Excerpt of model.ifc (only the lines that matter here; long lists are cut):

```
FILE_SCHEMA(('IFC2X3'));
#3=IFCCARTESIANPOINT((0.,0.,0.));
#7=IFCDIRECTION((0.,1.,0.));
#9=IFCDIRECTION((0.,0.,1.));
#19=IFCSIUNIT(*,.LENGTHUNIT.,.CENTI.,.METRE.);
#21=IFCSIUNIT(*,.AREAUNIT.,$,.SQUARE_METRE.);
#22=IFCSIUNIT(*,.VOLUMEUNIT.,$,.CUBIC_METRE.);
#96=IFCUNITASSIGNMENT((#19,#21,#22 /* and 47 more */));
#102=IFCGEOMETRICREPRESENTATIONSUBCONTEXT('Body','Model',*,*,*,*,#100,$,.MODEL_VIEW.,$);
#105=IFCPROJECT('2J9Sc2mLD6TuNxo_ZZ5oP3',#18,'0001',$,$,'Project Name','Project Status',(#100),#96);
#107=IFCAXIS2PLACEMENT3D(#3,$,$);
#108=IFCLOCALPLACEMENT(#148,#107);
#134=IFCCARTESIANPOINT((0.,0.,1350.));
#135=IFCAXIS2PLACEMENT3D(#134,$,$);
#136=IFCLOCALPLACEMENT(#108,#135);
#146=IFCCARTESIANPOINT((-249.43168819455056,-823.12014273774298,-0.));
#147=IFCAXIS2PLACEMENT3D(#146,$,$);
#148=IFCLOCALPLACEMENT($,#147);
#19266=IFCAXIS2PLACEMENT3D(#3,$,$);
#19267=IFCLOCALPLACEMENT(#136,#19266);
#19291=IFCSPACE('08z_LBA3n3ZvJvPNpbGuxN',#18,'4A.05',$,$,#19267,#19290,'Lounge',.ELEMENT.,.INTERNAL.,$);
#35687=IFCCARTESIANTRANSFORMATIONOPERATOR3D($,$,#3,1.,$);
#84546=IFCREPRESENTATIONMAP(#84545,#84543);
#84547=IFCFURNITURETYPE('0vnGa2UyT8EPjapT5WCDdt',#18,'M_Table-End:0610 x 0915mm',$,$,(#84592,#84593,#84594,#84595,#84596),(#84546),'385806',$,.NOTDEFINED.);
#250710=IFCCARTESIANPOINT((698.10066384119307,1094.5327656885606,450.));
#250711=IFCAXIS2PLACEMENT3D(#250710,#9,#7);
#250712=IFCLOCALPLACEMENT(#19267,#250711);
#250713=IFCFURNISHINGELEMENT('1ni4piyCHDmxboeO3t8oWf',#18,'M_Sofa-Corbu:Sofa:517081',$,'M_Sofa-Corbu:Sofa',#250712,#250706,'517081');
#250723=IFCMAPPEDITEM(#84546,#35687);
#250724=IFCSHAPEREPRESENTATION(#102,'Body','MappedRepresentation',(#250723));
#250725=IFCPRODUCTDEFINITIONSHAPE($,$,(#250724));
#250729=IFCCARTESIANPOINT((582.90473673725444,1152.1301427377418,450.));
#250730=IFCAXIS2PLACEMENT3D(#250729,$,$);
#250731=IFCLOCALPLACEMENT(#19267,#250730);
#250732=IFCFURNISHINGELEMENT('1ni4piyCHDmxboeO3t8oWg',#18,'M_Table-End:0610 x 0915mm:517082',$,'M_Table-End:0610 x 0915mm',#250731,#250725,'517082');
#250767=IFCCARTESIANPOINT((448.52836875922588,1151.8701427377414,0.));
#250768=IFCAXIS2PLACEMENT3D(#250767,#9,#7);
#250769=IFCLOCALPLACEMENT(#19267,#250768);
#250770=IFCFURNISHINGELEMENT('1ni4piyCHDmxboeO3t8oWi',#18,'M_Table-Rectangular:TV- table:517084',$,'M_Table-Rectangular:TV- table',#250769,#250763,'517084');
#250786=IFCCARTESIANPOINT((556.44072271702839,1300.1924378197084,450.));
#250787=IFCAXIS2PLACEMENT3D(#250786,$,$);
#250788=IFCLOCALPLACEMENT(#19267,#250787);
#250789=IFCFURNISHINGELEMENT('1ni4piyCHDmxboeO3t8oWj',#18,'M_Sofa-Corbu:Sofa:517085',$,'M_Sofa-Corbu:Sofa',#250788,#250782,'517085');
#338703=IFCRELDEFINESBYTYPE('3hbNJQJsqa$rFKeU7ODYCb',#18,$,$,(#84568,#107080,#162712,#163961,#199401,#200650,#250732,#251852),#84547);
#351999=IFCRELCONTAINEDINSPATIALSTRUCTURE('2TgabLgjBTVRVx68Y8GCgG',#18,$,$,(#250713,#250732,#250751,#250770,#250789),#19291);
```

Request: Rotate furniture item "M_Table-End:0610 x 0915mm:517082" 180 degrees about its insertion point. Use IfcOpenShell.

```python
import ifcopenshell
import ifcopenshell.api.geometry
import ifcopenshell.util.placement

model = ifcopenshell.open("model.ifc")

item = model.by_guid("1ni4piyCHDmxboeO3t8oWg")
matrix = ifcopenshell.util.placement.get_local_placement(item.ObjectPlacement)
matrix = matrix @ ifcopenshell.util.placement.rotation(180, "Z")
ifcopenshell.api.geometry.edit_object_placement(model, product=item, matrix=matrix, is_si=False)

print(ifcopenshell.util.placement.get_local_placement(item.ObjectPlacement).round(3) + 0.0)

model.write("model_v2.ifc")
```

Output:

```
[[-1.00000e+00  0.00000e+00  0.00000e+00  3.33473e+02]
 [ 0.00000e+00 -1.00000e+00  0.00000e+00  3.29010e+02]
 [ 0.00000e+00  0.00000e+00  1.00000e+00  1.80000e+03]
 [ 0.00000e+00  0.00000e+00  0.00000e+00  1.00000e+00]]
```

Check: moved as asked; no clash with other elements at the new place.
